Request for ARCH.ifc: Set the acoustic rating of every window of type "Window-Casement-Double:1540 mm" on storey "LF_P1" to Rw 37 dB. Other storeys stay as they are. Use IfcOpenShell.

First a look at what the model holds.

```python
import ifcopenshell
import ifcopenshell.util.element

model = ifcopenshell.open("ARCH.ifc")
print(model.schema)
storey = next(s for s in model.by_type("IfcBuildingStorey") if s.Name == "LF_P1")
windows = [e for e in ifcopenshell.util.element.get_decomposition(storey) if e.is_a("IfcWindow")]
seen = {}
for e in windows:
    element_type = ifcopenshell.util.element.get_type(e)
    key = (element_type.Name if element_type != e and element_type else None, ifcopenshell.util.element.get_pset(e, "Pset_WindowCommon", "AcousticRating"))
    seen[key] = seen.get(key, 0) + 1
for (name, value), count in sorted(seen.items(), key=str):
    print(count, "x", name, "|", value)
```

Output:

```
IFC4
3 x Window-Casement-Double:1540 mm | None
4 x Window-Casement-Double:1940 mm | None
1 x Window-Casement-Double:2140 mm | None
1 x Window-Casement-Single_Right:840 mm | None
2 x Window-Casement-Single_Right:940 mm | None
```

```python
import ifcopenshell
import ifcopenshell.api.pset
import ifcopenshell.util.element

model = ifcopenshell.open("ARCH.ifc")

storey = next(s for s in model.by_type("IfcBuildingStorey") if s.Name == "LF_P1")
windows = [e for e in ifcopenshell.util.element.get_decomposition(storey) if e.is_a("IfcWindow")]

count = 0
for e in windows:
    element_type = ifcopenshell.util.element.get_type(e)
    if element_type in (None, e) or element_type.Name != "Window-Casement-Double:1540 mm":
        continue
    # add_pset returns the element's existing set when there is one.
    pset = ifcopenshell.api.pset.add_pset(model, product=e, name="Pset_WindowCommon")
    ifcopenshell.api.pset.edit_pset(model, pset=pset, properties={"AcousticRating": "Rw 37 dB"})
    count += 1

print(count, "windows updated")

model.write("ARCH_updated.ifc")
```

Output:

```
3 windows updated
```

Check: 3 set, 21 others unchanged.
